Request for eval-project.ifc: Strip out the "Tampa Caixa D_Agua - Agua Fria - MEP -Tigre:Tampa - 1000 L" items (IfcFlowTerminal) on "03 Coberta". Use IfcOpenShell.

First a look at what the model holds.

```python
import ifcopenshell
import ifcopenshell.util.element

model = ifcopenshell.open("eval-project.ifc")
print(model.schema)
storey = next(s for s in model.by_type("IfcBuildingStorey") if s.Name == "03 Coberta")
terminals = [e for e in ifcopenshell.util.element.get_decomposition(storey) if e.is_a("IfcFlowTerminal")]
seen = {}
for e in terminals:
    element_type = ifcopenshell.util.element.get_type(e)
    name = element_type.Name if element_type not in (None, e) else None
    seen[name] = seen.get(name, 0) + 1
for name, count in sorted(seen.items(), key=str):
    print(count, "x", name)
```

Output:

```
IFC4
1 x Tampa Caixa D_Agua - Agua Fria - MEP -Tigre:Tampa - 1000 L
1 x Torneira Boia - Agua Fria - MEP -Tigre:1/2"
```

```python
import ifcopenshell
import ifcopenshell.api.root
import ifcopenshell.util.element

model = ifcopenshell.open("eval-project.ifc")

storey = next(s for s in model.by_type("IfcBuildingStorey") if s.Name == "03 Coberta")
terminals = [e for e in ifcopenshell.util.element.get_decomposition(storey) if e.is_a("IfcFlowTerminal")]
targets = [e for e in terminals if (t := ifcopenshell.util.element.get_type(e)) not in (None, e) and t.Name == "Tampa Caixa D_Agua - Agua Fria - MEP -Tigre:Tampa - 1000 L"]

for e in targets:
    ifcopenshell.api.root.remove_product(model, product=e)
print(len(targets), "removed")

model.write("eval-project_rev.ifc")
```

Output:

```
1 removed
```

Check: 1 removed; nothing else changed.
